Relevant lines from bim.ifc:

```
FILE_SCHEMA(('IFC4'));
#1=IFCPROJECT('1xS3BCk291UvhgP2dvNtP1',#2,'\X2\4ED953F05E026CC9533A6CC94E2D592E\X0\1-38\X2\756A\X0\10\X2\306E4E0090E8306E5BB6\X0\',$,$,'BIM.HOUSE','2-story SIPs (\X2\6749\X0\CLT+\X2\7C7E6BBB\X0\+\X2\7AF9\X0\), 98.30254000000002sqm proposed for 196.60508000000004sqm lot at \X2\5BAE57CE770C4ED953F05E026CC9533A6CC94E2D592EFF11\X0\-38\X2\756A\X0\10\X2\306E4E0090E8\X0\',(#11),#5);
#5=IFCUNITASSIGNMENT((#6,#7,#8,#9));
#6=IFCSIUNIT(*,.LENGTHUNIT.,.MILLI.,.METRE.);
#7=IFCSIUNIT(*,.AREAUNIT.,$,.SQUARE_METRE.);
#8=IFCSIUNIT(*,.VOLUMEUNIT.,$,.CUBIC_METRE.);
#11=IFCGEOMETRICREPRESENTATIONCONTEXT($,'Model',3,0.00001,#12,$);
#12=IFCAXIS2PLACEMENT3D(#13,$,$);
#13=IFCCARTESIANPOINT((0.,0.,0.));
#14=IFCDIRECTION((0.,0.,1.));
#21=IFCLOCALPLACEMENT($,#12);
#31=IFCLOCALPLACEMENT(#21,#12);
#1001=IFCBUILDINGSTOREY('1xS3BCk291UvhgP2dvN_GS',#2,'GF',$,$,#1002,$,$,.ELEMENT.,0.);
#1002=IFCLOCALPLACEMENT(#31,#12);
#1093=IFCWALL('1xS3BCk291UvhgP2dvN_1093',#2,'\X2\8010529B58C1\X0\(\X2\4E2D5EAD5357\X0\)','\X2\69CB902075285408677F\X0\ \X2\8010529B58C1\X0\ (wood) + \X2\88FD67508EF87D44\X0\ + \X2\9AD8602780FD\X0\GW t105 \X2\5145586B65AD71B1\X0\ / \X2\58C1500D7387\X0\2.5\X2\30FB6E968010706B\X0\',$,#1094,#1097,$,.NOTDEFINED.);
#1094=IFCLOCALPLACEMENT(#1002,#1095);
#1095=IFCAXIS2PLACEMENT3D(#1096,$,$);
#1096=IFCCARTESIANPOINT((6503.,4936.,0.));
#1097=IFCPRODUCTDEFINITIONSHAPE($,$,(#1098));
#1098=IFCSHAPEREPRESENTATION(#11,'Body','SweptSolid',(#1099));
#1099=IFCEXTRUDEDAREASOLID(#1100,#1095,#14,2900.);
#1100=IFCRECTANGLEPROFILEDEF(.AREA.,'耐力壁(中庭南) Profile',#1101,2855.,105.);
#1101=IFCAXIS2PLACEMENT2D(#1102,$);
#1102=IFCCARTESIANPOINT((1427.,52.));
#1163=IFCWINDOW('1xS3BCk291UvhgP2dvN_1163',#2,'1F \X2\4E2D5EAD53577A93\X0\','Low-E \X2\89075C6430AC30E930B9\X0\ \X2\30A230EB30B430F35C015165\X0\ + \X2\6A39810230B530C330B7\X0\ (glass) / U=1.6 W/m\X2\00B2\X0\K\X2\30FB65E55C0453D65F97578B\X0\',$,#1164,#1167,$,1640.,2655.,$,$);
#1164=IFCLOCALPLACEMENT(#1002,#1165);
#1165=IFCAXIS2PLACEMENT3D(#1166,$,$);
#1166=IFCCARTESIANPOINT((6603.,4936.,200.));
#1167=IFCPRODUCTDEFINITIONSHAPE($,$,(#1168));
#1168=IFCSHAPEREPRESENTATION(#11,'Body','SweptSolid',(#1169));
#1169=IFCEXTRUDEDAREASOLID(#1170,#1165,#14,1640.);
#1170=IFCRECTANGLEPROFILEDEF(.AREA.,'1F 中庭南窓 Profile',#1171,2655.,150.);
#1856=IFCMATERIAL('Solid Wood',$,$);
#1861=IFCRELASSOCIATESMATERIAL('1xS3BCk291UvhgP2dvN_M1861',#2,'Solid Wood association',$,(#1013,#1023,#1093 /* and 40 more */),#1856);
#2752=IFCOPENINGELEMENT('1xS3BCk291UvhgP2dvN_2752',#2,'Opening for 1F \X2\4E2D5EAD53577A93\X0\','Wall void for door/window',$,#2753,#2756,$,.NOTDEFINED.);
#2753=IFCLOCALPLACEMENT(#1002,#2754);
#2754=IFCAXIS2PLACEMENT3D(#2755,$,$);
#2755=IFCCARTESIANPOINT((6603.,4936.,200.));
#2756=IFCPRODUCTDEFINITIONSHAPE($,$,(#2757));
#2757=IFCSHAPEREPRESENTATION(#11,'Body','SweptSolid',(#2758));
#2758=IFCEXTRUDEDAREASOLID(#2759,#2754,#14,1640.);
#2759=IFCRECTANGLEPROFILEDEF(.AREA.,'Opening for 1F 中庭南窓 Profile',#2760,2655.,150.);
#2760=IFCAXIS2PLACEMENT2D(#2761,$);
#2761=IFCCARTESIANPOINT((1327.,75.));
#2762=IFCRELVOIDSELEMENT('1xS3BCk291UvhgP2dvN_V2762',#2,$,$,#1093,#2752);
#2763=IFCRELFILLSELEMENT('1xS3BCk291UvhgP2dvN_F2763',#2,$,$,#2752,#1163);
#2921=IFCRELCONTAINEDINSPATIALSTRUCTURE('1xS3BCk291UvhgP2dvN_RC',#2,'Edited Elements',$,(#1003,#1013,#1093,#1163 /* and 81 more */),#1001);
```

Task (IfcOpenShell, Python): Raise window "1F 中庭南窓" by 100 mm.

```python
import numpy as np
import ifcopenshell
import ifcopenshell.api.geometry
import ifcopenshell.util.placement
import ifcopenshell.util.unit

model = ifcopenshell.open("bim.ifc")
unit_scale = ifcopenshell.util.unit.calculate_unit_scale(model)

window = model.by_guid("1xS3BCk291UvhgP2dvN_1163")
opening = window.FillsVoids[0].RelatingOpeningElement
dz = 100.0

shift = np.array([0.0, 0.0, dz])
# The window is not placed relative to its opening, so move both.
for product in (opening, window):
    matrix = ifcopenshell.util.placement.get_local_placement(product.ObjectPlacement)
    matrix[:3, 3] += shift
    ifcopenshell.api.geometry.edit_object_placement(model, product=product, matrix=matrix, is_si=False)

print(f"moved by {dz * unit_scale:+.3f} m")

model.write("bim_edited.ifc")
```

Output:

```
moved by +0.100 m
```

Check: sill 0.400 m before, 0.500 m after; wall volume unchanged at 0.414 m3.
